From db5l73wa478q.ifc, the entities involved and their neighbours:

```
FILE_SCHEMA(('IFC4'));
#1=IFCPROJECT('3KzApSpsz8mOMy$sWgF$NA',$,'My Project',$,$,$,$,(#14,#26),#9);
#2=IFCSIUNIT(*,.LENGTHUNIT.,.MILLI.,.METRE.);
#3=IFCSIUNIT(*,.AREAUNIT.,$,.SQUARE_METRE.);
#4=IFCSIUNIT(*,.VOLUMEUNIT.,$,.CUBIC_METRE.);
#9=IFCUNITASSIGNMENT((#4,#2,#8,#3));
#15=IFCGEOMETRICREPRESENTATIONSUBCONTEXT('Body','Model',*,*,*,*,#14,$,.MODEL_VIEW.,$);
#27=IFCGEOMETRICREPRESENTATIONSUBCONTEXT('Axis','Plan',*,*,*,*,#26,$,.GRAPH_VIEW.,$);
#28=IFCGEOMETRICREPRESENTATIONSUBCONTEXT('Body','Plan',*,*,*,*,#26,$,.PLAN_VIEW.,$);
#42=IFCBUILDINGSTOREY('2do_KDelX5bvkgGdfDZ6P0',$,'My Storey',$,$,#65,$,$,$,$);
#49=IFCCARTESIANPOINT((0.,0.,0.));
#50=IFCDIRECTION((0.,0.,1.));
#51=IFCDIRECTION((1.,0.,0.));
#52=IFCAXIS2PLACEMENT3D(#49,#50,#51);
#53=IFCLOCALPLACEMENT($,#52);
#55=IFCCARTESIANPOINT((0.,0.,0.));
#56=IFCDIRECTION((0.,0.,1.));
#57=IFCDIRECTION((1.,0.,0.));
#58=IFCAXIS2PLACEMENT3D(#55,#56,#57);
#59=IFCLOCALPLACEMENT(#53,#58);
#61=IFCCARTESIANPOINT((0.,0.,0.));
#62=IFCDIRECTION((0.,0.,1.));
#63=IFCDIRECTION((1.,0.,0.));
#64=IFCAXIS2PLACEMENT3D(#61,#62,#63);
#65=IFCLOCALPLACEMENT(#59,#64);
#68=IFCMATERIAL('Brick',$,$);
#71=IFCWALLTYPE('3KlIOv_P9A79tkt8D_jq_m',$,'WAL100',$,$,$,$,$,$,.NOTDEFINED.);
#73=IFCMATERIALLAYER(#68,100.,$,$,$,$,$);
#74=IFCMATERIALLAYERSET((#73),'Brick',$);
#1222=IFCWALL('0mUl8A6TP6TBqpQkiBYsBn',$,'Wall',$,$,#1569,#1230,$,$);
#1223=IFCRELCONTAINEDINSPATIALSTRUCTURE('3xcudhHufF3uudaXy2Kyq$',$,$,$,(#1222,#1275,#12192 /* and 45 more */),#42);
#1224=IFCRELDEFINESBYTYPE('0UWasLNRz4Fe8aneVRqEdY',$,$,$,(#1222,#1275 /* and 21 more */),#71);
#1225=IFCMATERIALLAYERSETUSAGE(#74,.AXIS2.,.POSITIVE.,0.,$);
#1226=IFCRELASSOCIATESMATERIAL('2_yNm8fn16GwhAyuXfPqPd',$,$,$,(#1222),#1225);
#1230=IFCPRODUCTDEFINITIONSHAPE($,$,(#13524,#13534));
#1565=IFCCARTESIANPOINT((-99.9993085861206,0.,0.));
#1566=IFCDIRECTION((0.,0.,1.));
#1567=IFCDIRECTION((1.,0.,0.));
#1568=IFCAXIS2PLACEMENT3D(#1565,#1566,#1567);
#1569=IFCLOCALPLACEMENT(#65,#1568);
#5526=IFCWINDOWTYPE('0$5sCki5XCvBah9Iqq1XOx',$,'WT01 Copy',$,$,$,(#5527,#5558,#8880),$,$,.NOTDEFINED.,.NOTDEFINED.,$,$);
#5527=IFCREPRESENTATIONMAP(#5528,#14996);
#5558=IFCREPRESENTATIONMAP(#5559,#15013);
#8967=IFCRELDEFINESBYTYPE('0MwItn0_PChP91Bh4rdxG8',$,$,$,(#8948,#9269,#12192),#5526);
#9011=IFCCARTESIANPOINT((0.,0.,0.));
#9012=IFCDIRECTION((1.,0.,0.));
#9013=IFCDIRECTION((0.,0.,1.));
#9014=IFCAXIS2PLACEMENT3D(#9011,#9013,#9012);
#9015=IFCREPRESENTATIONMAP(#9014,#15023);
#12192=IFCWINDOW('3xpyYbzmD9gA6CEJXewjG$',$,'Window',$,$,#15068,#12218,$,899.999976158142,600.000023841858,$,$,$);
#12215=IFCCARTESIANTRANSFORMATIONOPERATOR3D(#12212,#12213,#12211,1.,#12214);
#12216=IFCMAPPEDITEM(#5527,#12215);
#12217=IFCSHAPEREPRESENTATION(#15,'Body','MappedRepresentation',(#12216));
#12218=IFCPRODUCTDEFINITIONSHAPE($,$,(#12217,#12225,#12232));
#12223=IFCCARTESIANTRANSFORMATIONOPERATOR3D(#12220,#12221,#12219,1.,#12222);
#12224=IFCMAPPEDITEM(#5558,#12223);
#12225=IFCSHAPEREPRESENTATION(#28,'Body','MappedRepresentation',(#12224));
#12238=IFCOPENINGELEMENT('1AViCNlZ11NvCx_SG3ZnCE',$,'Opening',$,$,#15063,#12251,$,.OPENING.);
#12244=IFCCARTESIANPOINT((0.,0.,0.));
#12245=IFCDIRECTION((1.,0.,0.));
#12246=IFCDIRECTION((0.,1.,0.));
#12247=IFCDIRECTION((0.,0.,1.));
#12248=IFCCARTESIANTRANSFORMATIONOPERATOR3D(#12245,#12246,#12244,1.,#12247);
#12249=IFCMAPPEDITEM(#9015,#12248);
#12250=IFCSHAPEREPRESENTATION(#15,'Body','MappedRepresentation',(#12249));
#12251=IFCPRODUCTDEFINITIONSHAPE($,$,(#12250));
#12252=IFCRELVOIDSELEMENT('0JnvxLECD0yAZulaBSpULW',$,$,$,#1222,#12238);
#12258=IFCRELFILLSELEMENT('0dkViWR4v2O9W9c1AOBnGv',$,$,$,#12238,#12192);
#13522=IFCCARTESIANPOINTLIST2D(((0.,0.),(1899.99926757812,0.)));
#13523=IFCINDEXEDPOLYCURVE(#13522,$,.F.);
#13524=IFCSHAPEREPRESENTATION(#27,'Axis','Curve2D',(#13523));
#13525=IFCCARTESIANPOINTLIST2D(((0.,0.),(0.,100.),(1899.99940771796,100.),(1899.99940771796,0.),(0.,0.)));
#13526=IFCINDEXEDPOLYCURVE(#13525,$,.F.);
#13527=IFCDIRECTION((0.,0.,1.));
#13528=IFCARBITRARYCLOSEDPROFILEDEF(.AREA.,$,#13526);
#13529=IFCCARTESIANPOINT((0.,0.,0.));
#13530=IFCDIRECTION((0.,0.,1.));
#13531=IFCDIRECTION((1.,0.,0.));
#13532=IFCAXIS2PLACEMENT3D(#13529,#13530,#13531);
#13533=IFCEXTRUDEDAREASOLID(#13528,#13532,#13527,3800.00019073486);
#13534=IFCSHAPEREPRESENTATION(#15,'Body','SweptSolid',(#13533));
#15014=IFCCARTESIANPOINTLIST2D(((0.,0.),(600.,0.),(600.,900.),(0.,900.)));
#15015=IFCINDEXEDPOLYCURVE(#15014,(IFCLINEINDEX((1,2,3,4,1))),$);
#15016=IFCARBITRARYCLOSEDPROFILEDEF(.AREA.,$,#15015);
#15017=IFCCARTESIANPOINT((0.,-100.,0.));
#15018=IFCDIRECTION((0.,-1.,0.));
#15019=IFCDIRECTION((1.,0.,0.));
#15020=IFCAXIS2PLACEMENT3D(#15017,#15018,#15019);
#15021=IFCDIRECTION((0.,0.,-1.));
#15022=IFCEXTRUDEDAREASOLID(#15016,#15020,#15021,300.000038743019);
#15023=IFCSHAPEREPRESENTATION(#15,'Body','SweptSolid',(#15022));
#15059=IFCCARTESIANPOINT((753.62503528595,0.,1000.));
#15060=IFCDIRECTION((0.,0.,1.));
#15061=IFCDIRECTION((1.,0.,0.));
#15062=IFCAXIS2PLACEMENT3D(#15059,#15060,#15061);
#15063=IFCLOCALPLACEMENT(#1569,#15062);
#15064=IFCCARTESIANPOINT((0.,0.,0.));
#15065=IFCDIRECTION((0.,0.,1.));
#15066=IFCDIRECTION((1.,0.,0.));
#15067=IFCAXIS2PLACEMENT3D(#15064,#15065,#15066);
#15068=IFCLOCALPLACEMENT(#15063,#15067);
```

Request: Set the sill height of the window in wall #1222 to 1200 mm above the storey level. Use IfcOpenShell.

```python
import numpy as np
import ifcopenshell
import ifcopenshell.api.geometry
import ifcopenshell.geom
import ifcopenshell.util.element
import ifcopenshell.util.placement
import ifcopenshell.util.shape
import ifcopenshell.util.unit

model = ifcopenshell.open("db5l73wa478q.ifc")
unit_scale = ifcopenshell.util.unit.calculate_unit_scale(model)

window = model.by_guid("3xpyYbzmD9gA6CEJXewjG$")
opening = window.FillsVoids[0].RelatingOpeningElement
storey = ifcopenshell.util.element.get_container(window, ifc_class="IfcBuildingStorey")
level = ifcopenshell.util.placement.get_local_placement(storey.ObjectPlacement)[2, 3]

# The opening's origin need not be at the sill, so measure its lowest point.
shape = ifcopenshell.geom.create_shape(ifcopenshell.geom.settings(), opening)
bottom = ifcopenshell.util.shape.get_shape_bottom_elevation(shape, shape.geometry) / unit_scale
dz = level + 1200.0 - bottom

shift = np.array([0.0, 0.0, dz])
# The window is placed relative to its opening, so it follows when the opening moves.
matrix = ifcopenshell.util.placement.get_local_placement(opening.ObjectPlacement)
matrix[:3, 3] += shift
ifcopenshell.api.geometry.edit_object_placement(
    model, product=opening, matrix=matrix, is_si=False, should_transform_children=True
)

print(f"moved by {dz * unit_scale:+.3f} m")

model.write("db5l73wa478q_edited.ifc")
```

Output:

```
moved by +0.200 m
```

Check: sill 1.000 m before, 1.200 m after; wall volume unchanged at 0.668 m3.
